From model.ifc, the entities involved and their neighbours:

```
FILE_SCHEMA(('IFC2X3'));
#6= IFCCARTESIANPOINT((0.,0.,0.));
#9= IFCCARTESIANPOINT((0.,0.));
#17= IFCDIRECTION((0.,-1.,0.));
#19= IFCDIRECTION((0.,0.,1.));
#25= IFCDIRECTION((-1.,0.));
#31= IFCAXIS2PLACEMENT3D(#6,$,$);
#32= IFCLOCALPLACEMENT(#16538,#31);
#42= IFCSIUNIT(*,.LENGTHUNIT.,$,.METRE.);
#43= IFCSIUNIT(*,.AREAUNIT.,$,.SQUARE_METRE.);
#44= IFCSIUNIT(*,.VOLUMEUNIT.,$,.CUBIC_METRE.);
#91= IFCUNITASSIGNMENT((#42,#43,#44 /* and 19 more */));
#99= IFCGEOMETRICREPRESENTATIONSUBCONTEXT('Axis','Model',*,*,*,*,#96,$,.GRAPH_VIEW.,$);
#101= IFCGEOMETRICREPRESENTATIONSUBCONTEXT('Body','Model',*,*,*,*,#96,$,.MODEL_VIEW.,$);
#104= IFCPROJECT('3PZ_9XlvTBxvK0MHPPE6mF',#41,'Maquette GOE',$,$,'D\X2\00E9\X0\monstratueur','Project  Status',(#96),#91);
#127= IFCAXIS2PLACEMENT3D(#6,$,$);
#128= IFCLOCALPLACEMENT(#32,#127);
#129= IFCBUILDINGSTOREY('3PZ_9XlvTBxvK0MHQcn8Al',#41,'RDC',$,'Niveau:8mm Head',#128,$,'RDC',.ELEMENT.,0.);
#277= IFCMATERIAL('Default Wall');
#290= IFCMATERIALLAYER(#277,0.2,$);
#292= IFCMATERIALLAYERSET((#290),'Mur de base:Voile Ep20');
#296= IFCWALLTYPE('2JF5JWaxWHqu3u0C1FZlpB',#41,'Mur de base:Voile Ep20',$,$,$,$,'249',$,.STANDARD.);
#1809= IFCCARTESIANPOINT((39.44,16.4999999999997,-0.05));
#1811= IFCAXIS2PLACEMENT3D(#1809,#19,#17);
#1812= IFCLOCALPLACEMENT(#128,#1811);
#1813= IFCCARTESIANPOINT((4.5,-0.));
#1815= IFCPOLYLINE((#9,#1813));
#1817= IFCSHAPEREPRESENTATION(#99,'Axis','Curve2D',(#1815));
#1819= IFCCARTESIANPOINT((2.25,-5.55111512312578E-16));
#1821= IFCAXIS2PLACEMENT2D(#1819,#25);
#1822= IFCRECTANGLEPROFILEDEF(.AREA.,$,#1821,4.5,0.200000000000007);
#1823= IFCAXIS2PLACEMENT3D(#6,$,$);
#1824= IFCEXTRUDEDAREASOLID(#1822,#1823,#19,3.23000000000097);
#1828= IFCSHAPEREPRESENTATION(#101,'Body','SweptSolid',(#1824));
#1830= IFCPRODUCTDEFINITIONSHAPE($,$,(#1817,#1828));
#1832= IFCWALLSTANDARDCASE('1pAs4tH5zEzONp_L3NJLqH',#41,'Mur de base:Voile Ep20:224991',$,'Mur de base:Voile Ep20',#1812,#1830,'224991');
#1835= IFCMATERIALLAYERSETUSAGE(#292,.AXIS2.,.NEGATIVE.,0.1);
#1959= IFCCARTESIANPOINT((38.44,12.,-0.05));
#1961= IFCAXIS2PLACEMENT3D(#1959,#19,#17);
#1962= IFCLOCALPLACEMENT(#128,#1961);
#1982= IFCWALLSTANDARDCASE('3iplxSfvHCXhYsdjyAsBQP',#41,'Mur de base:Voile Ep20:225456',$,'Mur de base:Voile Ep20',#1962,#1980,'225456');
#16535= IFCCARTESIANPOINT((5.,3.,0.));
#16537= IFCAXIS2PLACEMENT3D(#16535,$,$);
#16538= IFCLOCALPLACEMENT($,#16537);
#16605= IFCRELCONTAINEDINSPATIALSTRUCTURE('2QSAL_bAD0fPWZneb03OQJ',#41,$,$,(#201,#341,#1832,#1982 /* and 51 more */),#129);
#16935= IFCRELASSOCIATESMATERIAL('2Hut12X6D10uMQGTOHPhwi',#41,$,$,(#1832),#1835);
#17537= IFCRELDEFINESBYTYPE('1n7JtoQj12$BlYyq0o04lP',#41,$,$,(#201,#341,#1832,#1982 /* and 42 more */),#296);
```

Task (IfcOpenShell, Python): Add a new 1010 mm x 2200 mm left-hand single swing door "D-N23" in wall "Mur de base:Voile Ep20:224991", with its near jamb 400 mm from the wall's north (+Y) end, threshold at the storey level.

```python
import numpy as np
import ifcopenshell
import ifcopenshell.api.feature
import ifcopenshell.api.geometry
import ifcopenshell.api.root
import ifcopenshell.api.spatial
import ifcopenshell.api.type
import ifcopenshell.geom
import ifcopenshell.util.element
import ifcopenshell.util.placement
import ifcopenshell.util.representation
import ifcopenshell.util.shape
import ifcopenshell.util.unit

model = ifcopenshell.open("model.ifc")
unit_scale = ifcopenshell.util.unit.calculate_unit_scale(model)
settings = ifcopenshell.geom.settings()


def volume(element):
    """Net volume in cubic metres, openings subtracted."""
    shape = ifcopenshell.geom.create_shape(settings, element)
    return ifcopenshell.util.shape.get_volume(shape.geometry)


wall = model.by_guid("1pAs4tH5zEzONp_L3NJLqH")
storey = ifcopenshell.util.element.get_container(wall, ifc_class="IfcBuildingStorey")
context = ifcopenshell.util.representation.get_context(model, "Model", "Body", "MODEL_VIEW")
before = volume(wall)

width, height, from_end, sill = 1.01, 2.2, 0.4, 0.0  # metres

# The wall runs along its own X axis, and the end named is its -X end.
wall_shape = ifcopenshell.geom.create_shape(settings, wall)
x, y, z = ifcopenshell.util.shape.get_vertices(wall_shape.geometry).T
start = x.min() + from_end
face, thickness = float(y.min()), float(y.max() - y.min())
wall_matrix = ifcopenshell.util.placement.get_local_placement(wall.ObjectPlacement)
level = ifcopenshell.util.placement.get_local_placement(storey.ObjectPlacement)[2, 3]


def in_wall(x, y):
    """Placement at x, y metres in the wall's axes, at sill height."""
    matrix = wall_matrix.copy()
    matrix[:, 3] = wall_matrix @ np.array([x / unit_scale, y / unit_scale, 0.0, 1.0])
    matrix[2, 3] = level + sill / unit_scale
    return matrix


# Opening: a box that overshoots both wall faces by 50 mm.
opening = ifcopenshell.api.root.create_entity(model, ifc_class="IfcOpeningElement")
box = ifcopenshell.api.geometry.add_wall_representation(
    model, context=context, length=width, height=height, thickness=thickness + 0.1
)
ifcopenshell.api.geometry.assign_representation(model, product=opening, representation=box)
ifcopenshell.api.geometry.edit_object_placement(model, product=opening, matrix=in_wall(start, face - 0.05), is_si=False)
ifcopenshell.api.feature.add_feature(model, feature=opening, element=wall)

door = ifcopenshell.api.root.create_entity(model, ifc_class="IfcDoor", name="D-N23")
door.OverallWidth, door.OverallHeight = width / unit_scale, height / unit_scale
body = ifcopenshell.api.geometry.add_door_representation(
    model,
    context=context,
    overall_width=door.OverallWidth,
    overall_height=door.OverallHeight,
    operation_type="SINGLE_SWING_LEFT",
    lining_properties={"LiningDepth": thickness / unit_scale, "ThresholdDepth": thickness / unit_scale},
)
ifcopenshell.api.geometry.assign_representation(model, product=door, representation=body)
ifcopenshell.api.spatial.assign_container(model, products=[door], relating_structure=storey)
fills = ifcopenshell.api.feature.add_filling(model, opening=opening, element=door)
fills.OwnerHistory = door.OwnerHistory  # required in IFC2X3

# IFC2X3 keeps the operation on the door style.
style = ifcopenshell.api.root.create_entity(model, ifc_class="IfcDoorStyle", name="D-N23")
style.OperationType, style.ConstructionType = "SINGLE_SWING_LEFT", "NOTDEFINED"
style.ParameterTakesPrecedence = style.Sizeable = False
ifcopenshell.api.type.assign_type(model, related_objects=[door], relating_type=style)

# The lining spans the wall, so the door starts at the wall face.
ifcopenshell.api.geometry.edit_object_placement(model, product=door, matrix=in_wall(start, face), is_si=False)

after = volume(wall)

print(f"wall volume {before:.3f} -> {after:.3f} m3")

model.write("model_v2.ifc")
```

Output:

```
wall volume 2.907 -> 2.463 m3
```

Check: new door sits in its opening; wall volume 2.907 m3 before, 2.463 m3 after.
